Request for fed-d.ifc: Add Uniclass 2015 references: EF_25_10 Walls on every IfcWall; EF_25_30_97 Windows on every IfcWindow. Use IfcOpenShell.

First a look at what the model holds.

```python
import ifcopenshell

model = ifcopenshell.open("fed-d.ifc")
print(model.schema)
print("classifications:", [c.Name for c in model.by_type("IfcClassification")])
for ifc_class in ("IfcDoor", "IfcRoof", "IfcStair", "IfcWall", "IfcWindow"):
    print(ifc_class, len(model.by_type(ifc_class)))
```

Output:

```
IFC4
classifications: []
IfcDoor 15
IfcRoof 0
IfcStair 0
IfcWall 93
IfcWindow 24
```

```python
import ifcopenshell
import ifcopenshell.api.classification

model = ifcopenshell.open("fed-d.ifc")

system = ifcopenshell.api.classification.add_classification(model, classification="Uniclass 2015")

codes = {
    "IfcWall": ("EF_25_10", "Walls"),
    "IfcWindow": ("EF_25_30_97", "Windows"),
}
for ifc_class, (code, name) in codes.items():
    products = model.by_type(ifc_class)
    ifcopenshell.api.classification.add_reference(
        model, products=products, classification=system, identification=code, name=name
    )
    print(code, len(products))

model.write("fed-d_v2.ifc")
```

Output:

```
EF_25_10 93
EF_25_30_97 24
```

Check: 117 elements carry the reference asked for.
